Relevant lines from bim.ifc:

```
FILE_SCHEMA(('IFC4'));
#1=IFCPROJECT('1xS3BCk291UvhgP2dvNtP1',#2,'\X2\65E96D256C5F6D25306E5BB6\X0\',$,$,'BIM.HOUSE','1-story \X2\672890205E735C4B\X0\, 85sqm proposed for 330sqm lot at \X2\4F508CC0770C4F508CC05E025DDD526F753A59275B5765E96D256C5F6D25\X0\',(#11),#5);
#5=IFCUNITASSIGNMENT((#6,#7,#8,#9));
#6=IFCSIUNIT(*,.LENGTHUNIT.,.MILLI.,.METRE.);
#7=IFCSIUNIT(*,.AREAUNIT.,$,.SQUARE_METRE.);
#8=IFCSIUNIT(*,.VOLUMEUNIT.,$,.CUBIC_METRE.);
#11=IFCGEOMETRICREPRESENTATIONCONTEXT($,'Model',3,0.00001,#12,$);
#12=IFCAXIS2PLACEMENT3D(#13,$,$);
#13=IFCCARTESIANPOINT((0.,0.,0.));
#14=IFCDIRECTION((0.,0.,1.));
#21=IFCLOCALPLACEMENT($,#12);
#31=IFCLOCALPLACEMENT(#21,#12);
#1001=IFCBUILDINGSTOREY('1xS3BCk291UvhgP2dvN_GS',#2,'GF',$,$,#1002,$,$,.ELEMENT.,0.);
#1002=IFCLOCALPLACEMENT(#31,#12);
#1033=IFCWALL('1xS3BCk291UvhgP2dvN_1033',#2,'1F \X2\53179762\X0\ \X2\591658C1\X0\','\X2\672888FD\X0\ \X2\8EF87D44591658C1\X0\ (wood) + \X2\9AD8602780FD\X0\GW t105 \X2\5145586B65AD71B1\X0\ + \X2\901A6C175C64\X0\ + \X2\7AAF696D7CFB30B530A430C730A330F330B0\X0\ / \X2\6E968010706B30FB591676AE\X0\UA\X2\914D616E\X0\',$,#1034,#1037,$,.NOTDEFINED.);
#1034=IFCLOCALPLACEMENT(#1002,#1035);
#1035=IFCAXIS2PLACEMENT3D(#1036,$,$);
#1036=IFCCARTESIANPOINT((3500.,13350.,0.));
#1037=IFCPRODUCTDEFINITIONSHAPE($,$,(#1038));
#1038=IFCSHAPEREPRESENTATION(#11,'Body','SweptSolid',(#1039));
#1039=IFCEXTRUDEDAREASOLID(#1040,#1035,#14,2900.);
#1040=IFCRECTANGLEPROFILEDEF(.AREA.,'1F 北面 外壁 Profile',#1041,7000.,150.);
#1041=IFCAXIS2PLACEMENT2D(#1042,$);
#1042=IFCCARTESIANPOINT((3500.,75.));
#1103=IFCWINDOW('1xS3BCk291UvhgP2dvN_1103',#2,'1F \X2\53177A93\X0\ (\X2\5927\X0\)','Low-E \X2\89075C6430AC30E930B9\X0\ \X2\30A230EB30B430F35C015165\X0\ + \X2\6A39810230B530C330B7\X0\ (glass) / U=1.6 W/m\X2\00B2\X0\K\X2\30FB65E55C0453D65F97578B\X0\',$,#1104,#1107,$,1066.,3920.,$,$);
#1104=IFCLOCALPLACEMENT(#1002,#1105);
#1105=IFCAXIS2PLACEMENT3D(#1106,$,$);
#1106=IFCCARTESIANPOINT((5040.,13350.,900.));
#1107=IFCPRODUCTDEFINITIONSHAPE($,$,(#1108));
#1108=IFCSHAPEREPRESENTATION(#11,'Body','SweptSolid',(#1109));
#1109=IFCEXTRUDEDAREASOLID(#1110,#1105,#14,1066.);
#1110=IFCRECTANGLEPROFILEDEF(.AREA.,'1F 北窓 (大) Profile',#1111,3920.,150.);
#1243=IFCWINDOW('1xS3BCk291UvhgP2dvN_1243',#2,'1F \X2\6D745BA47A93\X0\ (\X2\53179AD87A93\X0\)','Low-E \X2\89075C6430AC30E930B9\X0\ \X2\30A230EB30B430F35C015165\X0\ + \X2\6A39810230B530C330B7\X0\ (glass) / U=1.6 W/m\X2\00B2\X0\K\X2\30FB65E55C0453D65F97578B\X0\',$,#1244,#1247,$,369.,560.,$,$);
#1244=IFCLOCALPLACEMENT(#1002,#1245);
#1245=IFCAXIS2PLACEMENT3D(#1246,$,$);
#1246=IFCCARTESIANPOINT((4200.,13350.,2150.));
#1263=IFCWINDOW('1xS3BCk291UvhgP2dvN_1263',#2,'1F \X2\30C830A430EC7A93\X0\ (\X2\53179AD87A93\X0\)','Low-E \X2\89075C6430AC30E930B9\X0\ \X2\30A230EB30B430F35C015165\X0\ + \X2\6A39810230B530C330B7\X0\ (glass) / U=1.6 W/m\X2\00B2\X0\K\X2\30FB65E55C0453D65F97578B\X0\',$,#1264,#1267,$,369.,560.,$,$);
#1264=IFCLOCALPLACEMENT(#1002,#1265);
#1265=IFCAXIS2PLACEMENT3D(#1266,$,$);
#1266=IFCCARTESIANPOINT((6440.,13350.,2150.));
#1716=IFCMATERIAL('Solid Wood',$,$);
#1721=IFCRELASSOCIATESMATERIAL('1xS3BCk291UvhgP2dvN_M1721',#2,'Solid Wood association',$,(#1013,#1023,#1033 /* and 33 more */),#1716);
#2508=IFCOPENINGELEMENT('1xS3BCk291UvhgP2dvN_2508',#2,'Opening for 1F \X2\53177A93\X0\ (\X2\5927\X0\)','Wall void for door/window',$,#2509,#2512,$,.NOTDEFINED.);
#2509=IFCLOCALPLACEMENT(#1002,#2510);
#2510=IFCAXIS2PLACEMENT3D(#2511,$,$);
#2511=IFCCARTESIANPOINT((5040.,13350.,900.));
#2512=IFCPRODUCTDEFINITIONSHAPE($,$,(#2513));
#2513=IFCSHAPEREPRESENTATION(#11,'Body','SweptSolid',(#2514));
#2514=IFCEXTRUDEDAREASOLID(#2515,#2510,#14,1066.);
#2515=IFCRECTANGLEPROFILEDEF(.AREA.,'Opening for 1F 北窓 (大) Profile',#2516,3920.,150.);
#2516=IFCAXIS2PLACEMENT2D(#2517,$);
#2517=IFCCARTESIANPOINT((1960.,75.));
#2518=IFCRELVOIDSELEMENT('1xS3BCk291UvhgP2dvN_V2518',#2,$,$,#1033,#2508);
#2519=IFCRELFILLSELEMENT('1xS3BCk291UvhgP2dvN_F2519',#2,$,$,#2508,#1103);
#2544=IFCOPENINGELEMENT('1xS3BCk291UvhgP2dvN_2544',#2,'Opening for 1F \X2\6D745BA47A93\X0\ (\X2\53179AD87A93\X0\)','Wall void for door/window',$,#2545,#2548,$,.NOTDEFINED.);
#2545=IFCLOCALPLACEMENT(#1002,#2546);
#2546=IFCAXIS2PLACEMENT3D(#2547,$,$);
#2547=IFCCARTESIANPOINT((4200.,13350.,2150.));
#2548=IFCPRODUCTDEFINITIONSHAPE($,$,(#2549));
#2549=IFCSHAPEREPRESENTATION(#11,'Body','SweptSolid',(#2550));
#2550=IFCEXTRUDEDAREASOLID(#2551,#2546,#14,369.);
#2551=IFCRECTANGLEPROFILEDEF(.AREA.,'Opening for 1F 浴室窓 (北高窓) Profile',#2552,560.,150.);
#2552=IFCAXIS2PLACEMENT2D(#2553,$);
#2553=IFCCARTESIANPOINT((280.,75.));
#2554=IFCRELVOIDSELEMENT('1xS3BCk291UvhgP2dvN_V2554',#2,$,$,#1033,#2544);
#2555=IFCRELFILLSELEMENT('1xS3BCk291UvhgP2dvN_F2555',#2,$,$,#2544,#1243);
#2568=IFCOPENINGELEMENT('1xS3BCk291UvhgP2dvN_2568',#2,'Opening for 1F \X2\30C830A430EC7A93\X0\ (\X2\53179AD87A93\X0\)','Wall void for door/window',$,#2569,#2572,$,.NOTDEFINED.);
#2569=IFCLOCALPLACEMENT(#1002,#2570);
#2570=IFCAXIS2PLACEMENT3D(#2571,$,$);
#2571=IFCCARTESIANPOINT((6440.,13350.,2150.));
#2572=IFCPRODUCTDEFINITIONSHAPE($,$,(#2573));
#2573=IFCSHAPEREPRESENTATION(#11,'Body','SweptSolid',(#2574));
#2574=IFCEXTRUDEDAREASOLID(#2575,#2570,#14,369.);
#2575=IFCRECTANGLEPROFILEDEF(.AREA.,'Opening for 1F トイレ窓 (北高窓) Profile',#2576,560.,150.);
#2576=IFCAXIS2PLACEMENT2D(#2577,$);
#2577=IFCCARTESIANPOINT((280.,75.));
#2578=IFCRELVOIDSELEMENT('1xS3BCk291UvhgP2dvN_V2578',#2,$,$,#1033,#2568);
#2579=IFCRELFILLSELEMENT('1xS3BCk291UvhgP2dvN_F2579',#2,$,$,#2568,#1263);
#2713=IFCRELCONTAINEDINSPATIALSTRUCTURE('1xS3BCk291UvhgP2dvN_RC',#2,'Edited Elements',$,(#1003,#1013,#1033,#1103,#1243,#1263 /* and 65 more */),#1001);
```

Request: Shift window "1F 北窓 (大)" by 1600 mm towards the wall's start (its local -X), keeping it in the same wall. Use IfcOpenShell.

```python
import ifcopenshell
import ifcopenshell.api.geometry
import ifcopenshell.util.placement

model = ifcopenshell.open("bim.ifc")

window = model.by_guid("1xS3BCk291UvhgP2dvN_1103")
opening = window.FillsVoids[0].RelatingOpeningElement
wall = opening.VoidsElements[0].RelatingBuildingElement

wall_matrix = ifcopenshell.util.placement.get_local_placement(wall.ObjectPlacement)
shift = wall_matrix[:3, 0] * -1600.0
before = ifcopenshell.util.placement.get_local_placement(window.ObjectPlacement)[:3, 3].copy()

# The window is not placed relative to its opening, so move both.
for product in (opening, window):
    matrix = ifcopenshell.util.placement.get_local_placement(product.ObjectPlacement)
    matrix[:3, 3] += shift
    ifcopenshell.api.geometry.edit_object_placement(model, product=product, matrix=matrix, is_si=False)

after = ifcopenshell.util.placement.get_local_placement(window.ObjectPlacement)[:3, 3]
print("window moved by", (after - before).round(3) + 0.0)

model.write("bim_updated.ifc")
```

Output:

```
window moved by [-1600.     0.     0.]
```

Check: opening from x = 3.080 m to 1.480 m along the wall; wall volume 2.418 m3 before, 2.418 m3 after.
